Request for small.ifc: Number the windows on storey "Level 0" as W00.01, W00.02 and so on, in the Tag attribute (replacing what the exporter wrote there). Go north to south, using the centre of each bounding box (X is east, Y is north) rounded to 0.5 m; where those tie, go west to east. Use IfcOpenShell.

First a look at what the model holds.

```python
import ifcopenshell
import ifcopenshell.util.element
import ifcopenshell.util.placement

model = ifcopenshell.open("small.ifc")
print(model.schema)
storey = next(s for s in model.by_type("IfcBuildingStorey") if s.Name == "Level 0")
windows = [e for e in ifcopenshell.util.element.get_decomposition(storey) if e.is_a("IfcWindow")]
for e in sorted(windows, key=lambda e: e.id()):
    origin = ifcopenshell.util.placement.get_local_placement(e.ObjectPlacement)[:3, 3]
    print(e.id(), e.Tag, e.Name, origin.round(2) + 0.0, sep=" | ")
```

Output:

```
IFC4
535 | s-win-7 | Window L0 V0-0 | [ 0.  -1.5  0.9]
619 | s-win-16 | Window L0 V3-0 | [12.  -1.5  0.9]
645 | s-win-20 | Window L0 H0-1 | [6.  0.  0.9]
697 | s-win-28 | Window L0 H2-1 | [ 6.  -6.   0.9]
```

```python
import ifcopenshell
import ifcopenshell.geom
import ifcopenshell.util.element
import ifcopenshell.util.shape

model = ifcopenshell.open("small.ifc")
settings = ifcopenshell.geom.settings()
settings.set("use-world-coords", True)


def centre(element):
    shape = ifcopenshell.geom.create_shape(settings, element)
    return ifcopenshell.util.shape.get_bbox_centroid(shape.geometry)


storey = next(s for s in model.by_type("IfcBuildingStorey") if s.Name == "Level 0")
windows = [e for e in ifcopenshell.util.element.get_decomposition(storey) if e.is_a("IfcWindow")]

# Insertion points can sit at a corner or the storey origin, so sort by the geometry (in metres).
centres = {e: centre(e) for e in windows}
windows.sort(key=lambda e: (-round(centres[e][1] / 0.5), centres[e][0]))

for i, e in enumerate(windows, start=1):
    number = f"W00.{i:02d}"
    e.Tag = number
    print(e.id(), number)

model.write("small-out.ifc")
```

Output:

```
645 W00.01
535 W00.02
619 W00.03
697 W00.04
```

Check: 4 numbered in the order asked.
